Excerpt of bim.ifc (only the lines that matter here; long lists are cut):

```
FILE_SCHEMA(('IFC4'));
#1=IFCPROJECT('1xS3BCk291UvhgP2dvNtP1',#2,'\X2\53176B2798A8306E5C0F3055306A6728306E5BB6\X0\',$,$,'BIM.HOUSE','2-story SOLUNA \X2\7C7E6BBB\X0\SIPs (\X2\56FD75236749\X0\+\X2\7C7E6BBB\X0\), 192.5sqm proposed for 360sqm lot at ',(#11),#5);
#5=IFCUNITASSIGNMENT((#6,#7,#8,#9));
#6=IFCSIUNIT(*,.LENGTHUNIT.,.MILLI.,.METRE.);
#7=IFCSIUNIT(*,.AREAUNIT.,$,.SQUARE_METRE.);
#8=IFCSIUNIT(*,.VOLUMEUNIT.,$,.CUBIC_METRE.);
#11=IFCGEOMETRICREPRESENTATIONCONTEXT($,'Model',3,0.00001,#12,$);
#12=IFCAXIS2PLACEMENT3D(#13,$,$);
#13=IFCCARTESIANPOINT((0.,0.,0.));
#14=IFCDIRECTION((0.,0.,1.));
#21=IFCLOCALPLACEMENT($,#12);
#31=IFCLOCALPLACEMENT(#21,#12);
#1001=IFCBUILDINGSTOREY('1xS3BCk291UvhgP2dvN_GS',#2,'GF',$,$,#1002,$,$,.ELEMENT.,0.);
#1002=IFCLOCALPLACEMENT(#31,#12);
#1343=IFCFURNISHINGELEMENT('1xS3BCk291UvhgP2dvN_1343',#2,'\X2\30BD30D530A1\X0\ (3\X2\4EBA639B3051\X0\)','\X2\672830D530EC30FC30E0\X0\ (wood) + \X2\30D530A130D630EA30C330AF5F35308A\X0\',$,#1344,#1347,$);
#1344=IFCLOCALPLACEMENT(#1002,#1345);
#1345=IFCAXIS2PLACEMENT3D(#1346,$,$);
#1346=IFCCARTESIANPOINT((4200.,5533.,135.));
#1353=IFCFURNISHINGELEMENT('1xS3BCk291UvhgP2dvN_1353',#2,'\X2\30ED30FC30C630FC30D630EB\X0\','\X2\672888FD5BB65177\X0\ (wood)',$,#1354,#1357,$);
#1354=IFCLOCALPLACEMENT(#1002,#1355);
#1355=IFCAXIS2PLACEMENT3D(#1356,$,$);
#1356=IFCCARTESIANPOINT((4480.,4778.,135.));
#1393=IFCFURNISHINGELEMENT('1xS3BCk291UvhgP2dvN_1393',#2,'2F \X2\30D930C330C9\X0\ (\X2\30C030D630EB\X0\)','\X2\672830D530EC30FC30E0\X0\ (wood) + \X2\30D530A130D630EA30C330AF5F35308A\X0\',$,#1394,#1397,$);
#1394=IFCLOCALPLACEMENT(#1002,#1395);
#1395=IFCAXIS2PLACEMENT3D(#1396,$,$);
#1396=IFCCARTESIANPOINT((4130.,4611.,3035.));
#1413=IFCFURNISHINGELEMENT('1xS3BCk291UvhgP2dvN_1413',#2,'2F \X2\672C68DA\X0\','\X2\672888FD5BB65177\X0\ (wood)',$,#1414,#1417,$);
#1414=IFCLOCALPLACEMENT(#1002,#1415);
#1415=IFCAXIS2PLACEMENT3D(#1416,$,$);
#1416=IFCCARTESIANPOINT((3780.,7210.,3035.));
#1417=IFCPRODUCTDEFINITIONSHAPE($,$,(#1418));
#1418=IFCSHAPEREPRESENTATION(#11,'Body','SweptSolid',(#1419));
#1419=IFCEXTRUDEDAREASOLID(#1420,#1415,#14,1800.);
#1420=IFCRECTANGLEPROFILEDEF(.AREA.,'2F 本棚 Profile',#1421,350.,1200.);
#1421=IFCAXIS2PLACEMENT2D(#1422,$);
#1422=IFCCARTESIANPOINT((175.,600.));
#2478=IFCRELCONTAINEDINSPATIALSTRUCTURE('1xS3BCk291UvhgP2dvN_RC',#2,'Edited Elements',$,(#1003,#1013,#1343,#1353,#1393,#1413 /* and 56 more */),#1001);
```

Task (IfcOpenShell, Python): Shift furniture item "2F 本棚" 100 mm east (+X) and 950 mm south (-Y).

```python
import ifcopenshell
import ifcopenshell.api.geometry
import ifcopenshell.util.placement
import ifcopenshell.util.unit

model = ifcopenshell.open("bim.ifc")
unit_scale = ifcopenshell.util.unit.calculate_unit_scale(model)

item = model.by_guid("1xS3BCk291UvhgP2dvN_1413")
matrix = ifcopenshell.util.placement.get_local_placement(item.ObjectPlacement)
matrix[0, 3] += 0.1 / unit_scale
matrix[1, 3] -= 0.95 / unit_scale
ifcopenshell.api.geometry.edit_object_placement(model, product=item, matrix=matrix, is_si=False)

print(ifcopenshell.util.placement.get_local_placement(item.ObjectPlacement).round(3) + 0.0)

model.write("bim_rev.ifc")
```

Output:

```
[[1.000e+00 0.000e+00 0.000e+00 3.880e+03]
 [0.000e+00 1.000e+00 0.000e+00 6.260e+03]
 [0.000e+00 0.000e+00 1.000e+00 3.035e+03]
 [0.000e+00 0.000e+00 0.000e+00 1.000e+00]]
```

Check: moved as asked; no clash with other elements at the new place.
